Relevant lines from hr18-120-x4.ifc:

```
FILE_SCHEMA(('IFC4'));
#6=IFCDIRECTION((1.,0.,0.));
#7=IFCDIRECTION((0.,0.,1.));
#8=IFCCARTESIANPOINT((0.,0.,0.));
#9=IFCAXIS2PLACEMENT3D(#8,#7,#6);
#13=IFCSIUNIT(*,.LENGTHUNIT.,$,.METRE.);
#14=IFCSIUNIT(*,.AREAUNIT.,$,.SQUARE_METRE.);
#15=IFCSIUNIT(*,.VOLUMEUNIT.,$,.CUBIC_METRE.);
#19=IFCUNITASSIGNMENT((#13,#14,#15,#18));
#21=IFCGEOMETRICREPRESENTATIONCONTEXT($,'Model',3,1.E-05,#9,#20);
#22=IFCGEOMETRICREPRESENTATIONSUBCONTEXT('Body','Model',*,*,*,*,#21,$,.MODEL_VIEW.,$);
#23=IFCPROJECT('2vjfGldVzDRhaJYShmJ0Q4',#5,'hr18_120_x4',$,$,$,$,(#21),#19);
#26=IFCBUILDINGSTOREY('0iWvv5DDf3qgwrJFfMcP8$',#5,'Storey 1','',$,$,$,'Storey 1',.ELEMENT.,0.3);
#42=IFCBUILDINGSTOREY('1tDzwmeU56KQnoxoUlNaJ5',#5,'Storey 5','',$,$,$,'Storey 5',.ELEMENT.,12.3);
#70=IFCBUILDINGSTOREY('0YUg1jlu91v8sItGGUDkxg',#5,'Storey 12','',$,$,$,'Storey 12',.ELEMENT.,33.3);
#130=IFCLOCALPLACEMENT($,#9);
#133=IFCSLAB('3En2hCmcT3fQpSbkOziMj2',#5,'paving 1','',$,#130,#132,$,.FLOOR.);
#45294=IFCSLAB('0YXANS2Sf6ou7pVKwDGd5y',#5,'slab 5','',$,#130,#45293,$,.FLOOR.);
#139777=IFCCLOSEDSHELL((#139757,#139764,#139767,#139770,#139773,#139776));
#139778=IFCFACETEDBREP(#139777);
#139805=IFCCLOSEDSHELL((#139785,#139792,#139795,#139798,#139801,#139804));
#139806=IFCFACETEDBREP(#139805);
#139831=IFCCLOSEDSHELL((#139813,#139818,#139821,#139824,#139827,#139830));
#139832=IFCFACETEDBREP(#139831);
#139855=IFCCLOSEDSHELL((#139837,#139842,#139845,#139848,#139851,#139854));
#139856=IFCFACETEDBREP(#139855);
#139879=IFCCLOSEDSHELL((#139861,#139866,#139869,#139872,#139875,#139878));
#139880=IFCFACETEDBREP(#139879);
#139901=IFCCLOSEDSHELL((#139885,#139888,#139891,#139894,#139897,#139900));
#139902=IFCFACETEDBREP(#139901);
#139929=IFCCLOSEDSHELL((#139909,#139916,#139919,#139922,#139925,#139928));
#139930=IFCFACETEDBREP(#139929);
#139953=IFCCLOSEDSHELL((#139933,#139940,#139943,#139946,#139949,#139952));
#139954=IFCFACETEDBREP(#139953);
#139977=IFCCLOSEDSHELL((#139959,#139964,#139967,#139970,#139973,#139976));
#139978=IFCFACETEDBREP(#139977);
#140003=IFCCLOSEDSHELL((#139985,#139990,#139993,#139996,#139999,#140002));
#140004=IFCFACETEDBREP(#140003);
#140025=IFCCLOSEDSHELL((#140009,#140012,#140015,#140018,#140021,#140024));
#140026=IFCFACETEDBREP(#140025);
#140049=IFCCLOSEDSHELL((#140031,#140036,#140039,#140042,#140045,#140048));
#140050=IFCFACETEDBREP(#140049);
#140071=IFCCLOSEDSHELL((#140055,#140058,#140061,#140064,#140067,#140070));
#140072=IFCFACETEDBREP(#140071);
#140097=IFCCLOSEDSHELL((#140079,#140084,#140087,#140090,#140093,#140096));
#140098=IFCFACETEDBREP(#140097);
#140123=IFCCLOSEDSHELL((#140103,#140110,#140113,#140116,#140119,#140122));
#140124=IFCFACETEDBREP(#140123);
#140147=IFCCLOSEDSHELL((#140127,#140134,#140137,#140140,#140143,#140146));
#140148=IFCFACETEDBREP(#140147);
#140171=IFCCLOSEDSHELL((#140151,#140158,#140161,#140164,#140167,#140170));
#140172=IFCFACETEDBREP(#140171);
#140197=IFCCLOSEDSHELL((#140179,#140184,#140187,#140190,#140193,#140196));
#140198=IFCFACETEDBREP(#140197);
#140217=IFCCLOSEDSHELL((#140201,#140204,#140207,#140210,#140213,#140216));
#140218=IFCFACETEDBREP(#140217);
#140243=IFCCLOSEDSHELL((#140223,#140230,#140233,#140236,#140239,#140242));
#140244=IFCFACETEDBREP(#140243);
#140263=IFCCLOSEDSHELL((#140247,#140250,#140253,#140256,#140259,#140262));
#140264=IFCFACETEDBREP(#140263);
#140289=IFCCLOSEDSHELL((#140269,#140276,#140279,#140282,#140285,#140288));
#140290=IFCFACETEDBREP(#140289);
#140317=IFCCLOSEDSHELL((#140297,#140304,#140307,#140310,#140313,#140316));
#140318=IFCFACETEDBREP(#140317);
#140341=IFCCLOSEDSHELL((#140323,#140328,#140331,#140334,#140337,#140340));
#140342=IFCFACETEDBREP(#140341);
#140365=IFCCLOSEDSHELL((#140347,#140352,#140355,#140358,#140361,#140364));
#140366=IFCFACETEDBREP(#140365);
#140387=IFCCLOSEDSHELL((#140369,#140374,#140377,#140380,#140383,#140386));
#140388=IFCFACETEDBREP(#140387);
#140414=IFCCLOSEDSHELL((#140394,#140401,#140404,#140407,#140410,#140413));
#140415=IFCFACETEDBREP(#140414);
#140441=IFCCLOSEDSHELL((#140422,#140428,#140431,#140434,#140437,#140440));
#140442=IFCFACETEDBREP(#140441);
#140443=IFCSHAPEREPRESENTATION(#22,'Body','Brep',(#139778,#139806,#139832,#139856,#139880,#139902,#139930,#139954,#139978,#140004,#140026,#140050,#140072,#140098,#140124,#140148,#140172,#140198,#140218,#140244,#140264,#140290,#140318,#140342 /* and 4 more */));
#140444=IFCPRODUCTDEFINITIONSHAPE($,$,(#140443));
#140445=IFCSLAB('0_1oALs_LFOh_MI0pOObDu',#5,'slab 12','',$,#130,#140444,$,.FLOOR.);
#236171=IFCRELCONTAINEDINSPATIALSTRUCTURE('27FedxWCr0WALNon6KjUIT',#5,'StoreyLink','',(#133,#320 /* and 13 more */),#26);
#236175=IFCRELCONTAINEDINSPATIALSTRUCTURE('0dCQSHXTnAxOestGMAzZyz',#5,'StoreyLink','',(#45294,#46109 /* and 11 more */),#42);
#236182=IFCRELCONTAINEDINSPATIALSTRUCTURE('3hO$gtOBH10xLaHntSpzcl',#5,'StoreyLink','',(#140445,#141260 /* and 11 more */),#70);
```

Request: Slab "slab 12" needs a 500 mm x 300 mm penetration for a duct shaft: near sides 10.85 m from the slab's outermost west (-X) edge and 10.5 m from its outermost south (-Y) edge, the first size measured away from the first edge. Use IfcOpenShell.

```python
import numpy as np
import ifcopenshell
import ifcopenshell.api.feature
import ifcopenshell.api.geometry
import ifcopenshell.api.root
import ifcopenshell.geom
import ifcopenshell.util.placement
import ifcopenshell.util.representation
import ifcopenshell.util.shape
import ifcopenshell.util.unit

model = ifcopenshell.open("hr18-120-x4.ifc")
unit_scale = ifcopenshell.util.unit.calculate_unit_scale(model)
settings = ifcopenshell.geom.settings()


def volume(element):
    """Net volume in cubic metres, openings subtracted."""
    shape = ifcopenshell.geom.create_shape(settings, element)
    return ifcopenshell.util.shape.get_volume(shape.geometry)


slab = model.by_guid("0_1oALs_LFOh_MI0pOObDu")
before = volume(slab)

# Extent in the slab's own axes, in metres. The edges named are its -X and -Y sides.
slab_shape = ifcopenshell.geom.create_shape(settings, slab)
vertices = ifcopenshell.util.shape.get_vertices(slab_shape.geometry)
x_min, y_min, bottom = vertices.min(axis=0)
top = vertices[:, 2].max()

opening = ifcopenshell.api.root.create_entity(model, ifc_class="IfcOpeningElement", name="Duct shaft opening", predefined_type="OPENING")
context = ifcopenshell.util.representation.get_context(model, "Model", "Body", "MODEL_VIEW")
width, depth = 0.5, 0.3
outline = [(0.0, 0.0), (width, 0.0), (width, depth), (0.0, depth), (0.0, 0.0)]
# Overshoot both faces by 50 mm so the cut is clean.
shape = ifcopenshell.api.geometry.add_slab_representation(
    model, context=context, depth=top - bottom + 0.1, polyline=outline
)
ifcopenshell.api.geometry.assign_representation(model, product=opening, representation=shape)

matrix = ifcopenshell.util.placement.get_local_placement(slab.ObjectPlacement)
matrix[:, 3] = matrix @ np.append(np.array([x_min + 10.85, y_min + 10.5, bottom - 0.05]) / unit_scale, 1.0)
ifcopenshell.api.geometry.edit_object_placement(model, product=opening, matrix=matrix, is_si=False)
ifcopenshell.api.feature.add_feature(model, feature=opening, element=slab)

after = volume(slab)

print(f"slab volume {before:.3f} -> {after:.3f} m3")

model.write("hr18-120-x4_updated.ifc")
```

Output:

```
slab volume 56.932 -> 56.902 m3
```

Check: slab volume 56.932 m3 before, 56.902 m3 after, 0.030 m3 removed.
